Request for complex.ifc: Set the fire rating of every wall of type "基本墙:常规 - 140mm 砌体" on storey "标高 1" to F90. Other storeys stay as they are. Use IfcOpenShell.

First a look at what the model holds.

```python
import ifcopenshell
import ifcopenshell.util.element

model = ifcopenshell.open("complex.ifc")
print(model.schema)
storey = next(s for s in model.by_type("IfcBuildingStorey") if s.Name == "标高 1")
walls = [e for e in ifcopenshell.util.element.get_decomposition(storey) if e.is_a("IfcWall")]
seen = {}
for e in walls:
    element_type = ifcopenshell.util.element.get_type(e)
    key = (element_type.Name if element_type != e and element_type else None, ifcopenshell.util.element.get_pset(e, "Pset_WallCommon", "FireRating"))
    seen[key] = seen.get(key, 0) + 1
for (name, value), count in sorted(seen.items(), key=str):
    print(count, "x", name, "|", value)
```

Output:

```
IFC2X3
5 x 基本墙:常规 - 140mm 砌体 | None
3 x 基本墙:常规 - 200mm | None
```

```python
import ifcopenshell
import ifcopenshell.api.pset
import ifcopenshell.util.element

model = ifcopenshell.open("complex.ifc")

storey = next(s for s in model.by_type("IfcBuildingStorey") if s.Name == "标高 1")
walls = [e for e in ifcopenshell.util.element.get_decomposition(storey) if e.is_a("IfcWall")]

count = 0
for e in walls:
    element_type = ifcopenshell.util.element.get_type(e)
    if element_type in (None, e) or element_type.Name != "基本墙:常规 - 140mm 砌体":
        continue
    # add_pset returns the element's existing set when there is one.
    pset = ifcopenshell.api.pset.add_pset(model, product=e, name="Pset_WallCommon")
    ifcopenshell.api.pset.edit_pset(model, pset=pset, properties={"FireRating": "F90"})
    count += 1

print(count, "walls updated")

model.write("complex-out.ifc")
```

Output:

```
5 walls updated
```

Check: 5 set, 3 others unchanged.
